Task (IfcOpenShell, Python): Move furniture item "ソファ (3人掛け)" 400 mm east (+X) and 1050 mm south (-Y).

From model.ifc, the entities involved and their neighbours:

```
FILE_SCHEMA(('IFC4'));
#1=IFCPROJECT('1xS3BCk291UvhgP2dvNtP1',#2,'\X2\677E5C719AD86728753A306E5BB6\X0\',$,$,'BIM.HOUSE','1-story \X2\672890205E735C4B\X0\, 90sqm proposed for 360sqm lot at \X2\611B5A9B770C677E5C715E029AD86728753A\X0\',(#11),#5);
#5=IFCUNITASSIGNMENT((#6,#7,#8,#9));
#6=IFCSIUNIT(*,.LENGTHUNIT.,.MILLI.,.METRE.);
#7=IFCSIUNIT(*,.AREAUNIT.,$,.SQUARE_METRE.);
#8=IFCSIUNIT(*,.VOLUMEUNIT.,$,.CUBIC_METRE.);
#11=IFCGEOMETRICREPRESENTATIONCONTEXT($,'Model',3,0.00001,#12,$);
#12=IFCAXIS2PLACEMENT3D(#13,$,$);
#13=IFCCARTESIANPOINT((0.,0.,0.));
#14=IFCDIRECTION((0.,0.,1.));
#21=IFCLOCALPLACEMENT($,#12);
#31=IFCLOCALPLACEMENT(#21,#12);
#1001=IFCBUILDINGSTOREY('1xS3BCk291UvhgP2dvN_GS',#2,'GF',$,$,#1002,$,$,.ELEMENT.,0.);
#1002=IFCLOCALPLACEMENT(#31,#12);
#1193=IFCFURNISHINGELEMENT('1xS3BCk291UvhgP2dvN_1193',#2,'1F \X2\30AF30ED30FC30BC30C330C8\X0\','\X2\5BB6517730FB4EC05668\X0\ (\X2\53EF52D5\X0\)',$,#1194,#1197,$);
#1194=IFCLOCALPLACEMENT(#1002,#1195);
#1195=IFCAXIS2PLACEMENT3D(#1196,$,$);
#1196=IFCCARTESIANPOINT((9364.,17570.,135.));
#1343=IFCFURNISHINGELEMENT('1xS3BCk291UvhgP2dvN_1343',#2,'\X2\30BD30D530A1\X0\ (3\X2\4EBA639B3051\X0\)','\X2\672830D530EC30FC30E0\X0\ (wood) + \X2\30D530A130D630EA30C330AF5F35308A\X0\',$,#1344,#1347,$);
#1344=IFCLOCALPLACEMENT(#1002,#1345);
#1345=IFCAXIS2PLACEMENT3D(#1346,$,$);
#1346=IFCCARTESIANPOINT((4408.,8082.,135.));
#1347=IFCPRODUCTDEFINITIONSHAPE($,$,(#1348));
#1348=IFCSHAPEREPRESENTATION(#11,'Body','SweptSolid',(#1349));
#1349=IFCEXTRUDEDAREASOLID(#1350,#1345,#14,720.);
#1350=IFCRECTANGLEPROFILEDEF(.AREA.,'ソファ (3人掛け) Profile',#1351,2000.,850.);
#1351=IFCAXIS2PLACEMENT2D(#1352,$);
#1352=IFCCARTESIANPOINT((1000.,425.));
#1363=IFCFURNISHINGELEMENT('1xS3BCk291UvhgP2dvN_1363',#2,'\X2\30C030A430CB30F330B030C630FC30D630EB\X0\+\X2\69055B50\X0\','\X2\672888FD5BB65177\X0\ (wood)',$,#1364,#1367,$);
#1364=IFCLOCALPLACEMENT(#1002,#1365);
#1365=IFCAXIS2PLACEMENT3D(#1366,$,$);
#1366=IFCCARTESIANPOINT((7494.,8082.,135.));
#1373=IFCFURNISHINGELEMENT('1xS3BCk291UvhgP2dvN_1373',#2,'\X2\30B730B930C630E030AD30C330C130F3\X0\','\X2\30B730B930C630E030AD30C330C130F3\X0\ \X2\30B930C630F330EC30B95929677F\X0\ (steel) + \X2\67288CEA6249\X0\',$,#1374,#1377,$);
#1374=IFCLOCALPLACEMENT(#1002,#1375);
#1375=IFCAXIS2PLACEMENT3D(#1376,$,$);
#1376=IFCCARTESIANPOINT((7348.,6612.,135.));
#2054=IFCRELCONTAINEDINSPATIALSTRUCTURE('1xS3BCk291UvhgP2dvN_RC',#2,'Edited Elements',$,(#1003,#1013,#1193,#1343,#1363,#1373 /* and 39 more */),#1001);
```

```python
import ifcopenshell
import ifcopenshell.api.geometry
import ifcopenshell.util.placement
import ifcopenshell.util.unit

model = ifcopenshell.open("model.ifc")
unit_scale = ifcopenshell.util.unit.calculate_unit_scale(model)

item = model.by_id(1343)
matrix = ifcopenshell.util.placement.get_local_placement(item.ObjectPlacement)
matrix[0, 3] += 0.4 / unit_scale
matrix[1, 3] -= 1.05 / unit_scale
ifcopenshell.api.geometry.edit_object_placement(model, product=item, matrix=matrix, is_si=False)

print(ifcopenshell.util.placement.get_local_placement(item.ObjectPlacement).round(3) + 0.0)

model.write("model_updated.ifc")
```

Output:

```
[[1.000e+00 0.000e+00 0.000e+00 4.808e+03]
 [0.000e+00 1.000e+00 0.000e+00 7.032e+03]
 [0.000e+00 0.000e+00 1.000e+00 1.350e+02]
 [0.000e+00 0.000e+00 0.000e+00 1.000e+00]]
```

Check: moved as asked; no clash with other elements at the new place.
